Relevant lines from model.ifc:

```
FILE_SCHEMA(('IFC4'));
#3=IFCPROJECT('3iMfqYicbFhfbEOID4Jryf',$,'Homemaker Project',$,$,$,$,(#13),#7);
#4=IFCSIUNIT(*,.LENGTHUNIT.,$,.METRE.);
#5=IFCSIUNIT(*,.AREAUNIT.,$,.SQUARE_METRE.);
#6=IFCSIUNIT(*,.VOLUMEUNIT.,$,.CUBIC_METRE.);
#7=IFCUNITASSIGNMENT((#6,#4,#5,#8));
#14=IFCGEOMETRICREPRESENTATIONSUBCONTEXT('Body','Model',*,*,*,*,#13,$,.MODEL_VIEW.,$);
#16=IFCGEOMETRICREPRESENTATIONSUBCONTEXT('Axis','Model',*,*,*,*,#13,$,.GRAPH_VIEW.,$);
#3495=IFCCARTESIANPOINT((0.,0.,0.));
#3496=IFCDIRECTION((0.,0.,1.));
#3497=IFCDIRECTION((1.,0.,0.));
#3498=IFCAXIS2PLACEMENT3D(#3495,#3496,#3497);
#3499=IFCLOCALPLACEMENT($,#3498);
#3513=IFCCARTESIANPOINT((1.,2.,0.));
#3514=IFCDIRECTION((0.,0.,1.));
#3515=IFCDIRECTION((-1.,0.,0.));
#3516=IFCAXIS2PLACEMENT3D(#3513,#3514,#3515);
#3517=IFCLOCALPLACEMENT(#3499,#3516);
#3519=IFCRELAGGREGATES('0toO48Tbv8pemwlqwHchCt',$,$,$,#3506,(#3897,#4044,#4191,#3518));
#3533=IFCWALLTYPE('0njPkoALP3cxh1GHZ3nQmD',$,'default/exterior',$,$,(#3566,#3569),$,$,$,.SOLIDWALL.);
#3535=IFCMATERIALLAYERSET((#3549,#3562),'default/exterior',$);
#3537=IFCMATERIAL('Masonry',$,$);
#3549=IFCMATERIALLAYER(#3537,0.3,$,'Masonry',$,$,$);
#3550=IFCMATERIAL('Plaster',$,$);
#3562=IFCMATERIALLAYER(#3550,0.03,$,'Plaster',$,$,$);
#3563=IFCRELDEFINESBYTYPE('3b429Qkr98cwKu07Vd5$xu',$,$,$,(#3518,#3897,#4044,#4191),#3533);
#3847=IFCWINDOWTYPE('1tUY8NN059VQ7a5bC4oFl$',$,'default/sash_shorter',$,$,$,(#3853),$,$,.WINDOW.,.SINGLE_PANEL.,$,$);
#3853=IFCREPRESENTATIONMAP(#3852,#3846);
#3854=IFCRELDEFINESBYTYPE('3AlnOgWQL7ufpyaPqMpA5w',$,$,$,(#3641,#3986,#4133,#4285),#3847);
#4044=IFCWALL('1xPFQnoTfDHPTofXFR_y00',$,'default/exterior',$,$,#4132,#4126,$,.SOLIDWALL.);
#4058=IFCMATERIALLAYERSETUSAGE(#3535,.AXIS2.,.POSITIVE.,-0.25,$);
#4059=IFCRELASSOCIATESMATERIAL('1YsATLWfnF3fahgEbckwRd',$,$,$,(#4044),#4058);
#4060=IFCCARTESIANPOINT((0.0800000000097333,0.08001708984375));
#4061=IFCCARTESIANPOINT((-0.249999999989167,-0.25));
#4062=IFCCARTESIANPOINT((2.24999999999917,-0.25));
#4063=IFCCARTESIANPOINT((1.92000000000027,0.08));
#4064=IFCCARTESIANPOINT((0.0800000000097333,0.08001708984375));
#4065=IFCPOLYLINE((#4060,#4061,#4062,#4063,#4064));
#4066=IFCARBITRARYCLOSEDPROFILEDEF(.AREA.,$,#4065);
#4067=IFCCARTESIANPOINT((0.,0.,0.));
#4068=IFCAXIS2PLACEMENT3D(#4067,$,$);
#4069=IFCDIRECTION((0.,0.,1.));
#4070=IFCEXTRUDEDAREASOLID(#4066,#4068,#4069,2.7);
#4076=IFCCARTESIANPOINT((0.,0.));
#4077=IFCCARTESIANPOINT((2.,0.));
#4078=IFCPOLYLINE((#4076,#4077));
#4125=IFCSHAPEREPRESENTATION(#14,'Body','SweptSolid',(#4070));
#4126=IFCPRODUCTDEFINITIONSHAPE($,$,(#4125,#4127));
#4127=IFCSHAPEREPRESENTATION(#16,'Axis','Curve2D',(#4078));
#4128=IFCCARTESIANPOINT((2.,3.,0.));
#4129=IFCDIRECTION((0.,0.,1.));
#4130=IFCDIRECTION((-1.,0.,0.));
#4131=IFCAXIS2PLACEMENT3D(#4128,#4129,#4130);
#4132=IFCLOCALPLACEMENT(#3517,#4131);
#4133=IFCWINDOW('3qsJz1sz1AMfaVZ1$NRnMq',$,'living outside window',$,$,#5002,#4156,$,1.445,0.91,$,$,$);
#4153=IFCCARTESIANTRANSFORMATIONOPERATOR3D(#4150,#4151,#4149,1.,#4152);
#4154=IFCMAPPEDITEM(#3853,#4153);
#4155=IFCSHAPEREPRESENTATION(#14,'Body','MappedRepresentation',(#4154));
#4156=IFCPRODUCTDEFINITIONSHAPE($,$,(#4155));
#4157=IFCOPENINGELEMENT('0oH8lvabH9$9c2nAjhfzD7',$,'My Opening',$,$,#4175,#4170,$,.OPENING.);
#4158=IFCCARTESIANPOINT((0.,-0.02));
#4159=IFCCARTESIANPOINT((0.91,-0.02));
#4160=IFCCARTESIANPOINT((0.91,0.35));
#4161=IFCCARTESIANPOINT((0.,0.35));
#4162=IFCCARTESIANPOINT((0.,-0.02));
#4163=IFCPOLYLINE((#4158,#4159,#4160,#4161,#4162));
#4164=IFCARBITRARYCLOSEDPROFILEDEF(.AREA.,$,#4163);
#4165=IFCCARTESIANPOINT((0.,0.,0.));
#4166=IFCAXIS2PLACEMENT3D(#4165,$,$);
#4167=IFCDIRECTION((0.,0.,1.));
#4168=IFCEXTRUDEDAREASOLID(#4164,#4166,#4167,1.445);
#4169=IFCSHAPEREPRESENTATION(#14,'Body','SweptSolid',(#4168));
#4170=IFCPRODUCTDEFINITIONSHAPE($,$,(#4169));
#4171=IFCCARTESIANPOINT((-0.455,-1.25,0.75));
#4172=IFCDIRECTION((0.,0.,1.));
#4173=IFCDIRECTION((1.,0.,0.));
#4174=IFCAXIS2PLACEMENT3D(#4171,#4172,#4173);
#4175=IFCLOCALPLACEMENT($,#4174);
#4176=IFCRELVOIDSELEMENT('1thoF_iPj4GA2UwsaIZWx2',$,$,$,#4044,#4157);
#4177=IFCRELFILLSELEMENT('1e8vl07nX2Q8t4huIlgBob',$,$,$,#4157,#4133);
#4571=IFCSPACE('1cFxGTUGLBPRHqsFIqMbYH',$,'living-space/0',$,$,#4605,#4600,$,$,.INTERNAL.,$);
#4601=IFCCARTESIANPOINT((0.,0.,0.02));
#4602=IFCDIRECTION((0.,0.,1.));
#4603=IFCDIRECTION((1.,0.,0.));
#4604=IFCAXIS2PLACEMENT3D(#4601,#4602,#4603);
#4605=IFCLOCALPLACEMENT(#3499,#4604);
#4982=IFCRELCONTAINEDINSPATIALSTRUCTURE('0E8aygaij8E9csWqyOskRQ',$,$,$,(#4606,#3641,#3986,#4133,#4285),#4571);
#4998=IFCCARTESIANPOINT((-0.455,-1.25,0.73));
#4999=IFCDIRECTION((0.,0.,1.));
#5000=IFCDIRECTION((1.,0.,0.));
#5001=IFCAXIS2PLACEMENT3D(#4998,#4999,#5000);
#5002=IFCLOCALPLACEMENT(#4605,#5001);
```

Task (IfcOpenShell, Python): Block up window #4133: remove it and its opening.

```python
import ifcopenshell
import ifcopenshell.api.feature
import ifcopenshell.api.root
import ifcopenshell.geom
import ifcopenshell.util.shape

model = ifcopenshell.open("model.ifc")
settings = ifcopenshell.geom.settings()


def volume(element):
    """Net volume in cubic metres, openings subtracted."""
    shape = ifcopenshell.geom.create_shape(settings, element)
    return ifcopenshell.util.shape.get_volume(shape.geometry)


window = model.by_guid("3qsJz1sz1AMfaVZ1$NRnMq")
opening = window.FillsVoids[0].RelatingOpeningElement
wall = opening.VoidsElements[0].RelatingBuildingElement
before = volume(wall)

ifcopenshell.api.root.remove_product(model, product=window)
ifcopenshell.api.feature.remove_feature(model, feature=opening)

after = volume(wall)

print(f"wall volume {before:.3f} -> {after:.3f} m3")

model.write("model-out.ifc")
```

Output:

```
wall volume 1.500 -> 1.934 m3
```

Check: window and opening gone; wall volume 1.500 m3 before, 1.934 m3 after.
